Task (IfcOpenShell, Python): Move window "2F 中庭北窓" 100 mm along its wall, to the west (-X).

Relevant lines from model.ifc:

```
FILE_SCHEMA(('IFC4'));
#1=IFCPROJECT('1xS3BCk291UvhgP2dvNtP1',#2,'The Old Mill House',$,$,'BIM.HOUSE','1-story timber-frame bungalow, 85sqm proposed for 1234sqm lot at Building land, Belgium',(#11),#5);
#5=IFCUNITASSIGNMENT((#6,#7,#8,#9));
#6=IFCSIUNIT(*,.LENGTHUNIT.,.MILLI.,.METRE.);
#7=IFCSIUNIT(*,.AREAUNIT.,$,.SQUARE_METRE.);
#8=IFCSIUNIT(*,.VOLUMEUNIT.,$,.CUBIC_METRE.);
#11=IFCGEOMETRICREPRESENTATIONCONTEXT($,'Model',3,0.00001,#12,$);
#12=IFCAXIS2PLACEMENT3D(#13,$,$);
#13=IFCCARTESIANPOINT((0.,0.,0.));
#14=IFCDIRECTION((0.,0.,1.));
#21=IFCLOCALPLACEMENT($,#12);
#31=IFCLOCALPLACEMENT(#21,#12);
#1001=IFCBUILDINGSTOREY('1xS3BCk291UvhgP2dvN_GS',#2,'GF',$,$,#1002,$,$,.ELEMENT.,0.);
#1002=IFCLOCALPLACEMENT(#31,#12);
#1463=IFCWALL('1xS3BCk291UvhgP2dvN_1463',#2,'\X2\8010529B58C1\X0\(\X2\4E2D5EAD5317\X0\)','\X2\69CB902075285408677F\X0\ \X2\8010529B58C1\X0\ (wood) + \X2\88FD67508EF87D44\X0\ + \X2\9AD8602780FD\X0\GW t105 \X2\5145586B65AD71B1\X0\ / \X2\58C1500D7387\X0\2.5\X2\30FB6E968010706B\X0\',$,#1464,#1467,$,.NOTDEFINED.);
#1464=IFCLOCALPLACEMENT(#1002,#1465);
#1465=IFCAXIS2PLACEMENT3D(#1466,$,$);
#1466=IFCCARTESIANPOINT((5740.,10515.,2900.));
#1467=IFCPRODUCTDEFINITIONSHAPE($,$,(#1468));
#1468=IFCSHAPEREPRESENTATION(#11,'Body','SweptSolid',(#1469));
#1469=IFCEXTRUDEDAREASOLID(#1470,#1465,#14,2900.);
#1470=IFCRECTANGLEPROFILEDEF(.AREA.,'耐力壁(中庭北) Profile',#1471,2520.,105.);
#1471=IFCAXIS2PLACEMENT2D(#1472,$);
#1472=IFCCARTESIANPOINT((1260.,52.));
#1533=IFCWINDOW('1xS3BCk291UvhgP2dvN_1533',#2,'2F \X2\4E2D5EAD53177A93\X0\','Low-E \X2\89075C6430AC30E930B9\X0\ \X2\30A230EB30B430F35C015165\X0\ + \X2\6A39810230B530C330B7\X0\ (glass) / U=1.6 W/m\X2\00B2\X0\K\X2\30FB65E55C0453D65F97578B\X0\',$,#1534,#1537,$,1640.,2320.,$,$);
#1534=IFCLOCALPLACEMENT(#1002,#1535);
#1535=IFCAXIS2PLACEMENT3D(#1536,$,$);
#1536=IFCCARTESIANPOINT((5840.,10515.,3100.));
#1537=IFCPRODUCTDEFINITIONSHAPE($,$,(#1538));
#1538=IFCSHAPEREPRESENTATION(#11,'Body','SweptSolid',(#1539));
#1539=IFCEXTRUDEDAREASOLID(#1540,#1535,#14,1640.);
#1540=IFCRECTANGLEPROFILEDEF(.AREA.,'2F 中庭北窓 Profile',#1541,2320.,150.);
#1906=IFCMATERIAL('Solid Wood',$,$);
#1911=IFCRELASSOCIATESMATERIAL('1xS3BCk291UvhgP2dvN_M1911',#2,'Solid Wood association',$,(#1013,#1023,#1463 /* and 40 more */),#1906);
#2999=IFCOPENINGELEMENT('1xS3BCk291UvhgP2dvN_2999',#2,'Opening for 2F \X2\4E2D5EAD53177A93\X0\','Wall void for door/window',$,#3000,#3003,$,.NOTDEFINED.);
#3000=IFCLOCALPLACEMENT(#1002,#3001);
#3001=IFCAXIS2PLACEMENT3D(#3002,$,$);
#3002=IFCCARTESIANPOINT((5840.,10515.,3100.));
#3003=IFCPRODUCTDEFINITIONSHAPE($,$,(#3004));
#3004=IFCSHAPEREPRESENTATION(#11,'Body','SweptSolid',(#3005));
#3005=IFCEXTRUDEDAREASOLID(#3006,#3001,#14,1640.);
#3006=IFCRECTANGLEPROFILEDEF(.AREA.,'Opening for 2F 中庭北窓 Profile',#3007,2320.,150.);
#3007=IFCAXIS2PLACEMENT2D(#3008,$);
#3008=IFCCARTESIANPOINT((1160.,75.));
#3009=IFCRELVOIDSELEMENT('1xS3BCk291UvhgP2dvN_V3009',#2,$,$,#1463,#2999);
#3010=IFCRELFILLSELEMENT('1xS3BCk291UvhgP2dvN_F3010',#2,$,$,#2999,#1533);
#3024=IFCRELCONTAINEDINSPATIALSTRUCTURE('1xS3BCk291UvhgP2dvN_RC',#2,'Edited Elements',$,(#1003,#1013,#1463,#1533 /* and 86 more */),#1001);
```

```python
import ifcopenshell
import ifcopenshell.api.geometry
import ifcopenshell.util.placement
import ifcopenshell.util.unit

model = ifcopenshell.open("model.ifc")
unit_scale = ifcopenshell.util.unit.calculate_unit_scale(model)

window = model.by_guid("1xS3BCk291UvhgP2dvN_1533")
opening = window.FillsVoids[0].RelatingOpeningElement
wall = opening.VoidsElements[0].RelatingBuildingElement

wall_matrix = ifcopenshell.util.placement.get_local_placement(wall.ObjectPlacement)
shift = wall_matrix[:3, 0] * -0.1 / unit_scale
before = ifcopenshell.util.placement.get_local_placement(window.ObjectPlacement)[:3, 3].copy()

# The window is not placed relative to its opening, so move both.
for product in (opening, window):
    matrix = ifcopenshell.util.placement.get_local_placement(product.ObjectPlacement)
    matrix[:3, 3] += shift
    ifcopenshell.api.geometry.edit_object_placement(model, product=product, matrix=matrix, is_si=False)

after = ifcopenshell.util.placement.get_local_placement(window.ObjectPlacement)[:3, 3]
print("window moved by", (after - before).round(3) + 0.0)

model.write("model-out.ifc")
```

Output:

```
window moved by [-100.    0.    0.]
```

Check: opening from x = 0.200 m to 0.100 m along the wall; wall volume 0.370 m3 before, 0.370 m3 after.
